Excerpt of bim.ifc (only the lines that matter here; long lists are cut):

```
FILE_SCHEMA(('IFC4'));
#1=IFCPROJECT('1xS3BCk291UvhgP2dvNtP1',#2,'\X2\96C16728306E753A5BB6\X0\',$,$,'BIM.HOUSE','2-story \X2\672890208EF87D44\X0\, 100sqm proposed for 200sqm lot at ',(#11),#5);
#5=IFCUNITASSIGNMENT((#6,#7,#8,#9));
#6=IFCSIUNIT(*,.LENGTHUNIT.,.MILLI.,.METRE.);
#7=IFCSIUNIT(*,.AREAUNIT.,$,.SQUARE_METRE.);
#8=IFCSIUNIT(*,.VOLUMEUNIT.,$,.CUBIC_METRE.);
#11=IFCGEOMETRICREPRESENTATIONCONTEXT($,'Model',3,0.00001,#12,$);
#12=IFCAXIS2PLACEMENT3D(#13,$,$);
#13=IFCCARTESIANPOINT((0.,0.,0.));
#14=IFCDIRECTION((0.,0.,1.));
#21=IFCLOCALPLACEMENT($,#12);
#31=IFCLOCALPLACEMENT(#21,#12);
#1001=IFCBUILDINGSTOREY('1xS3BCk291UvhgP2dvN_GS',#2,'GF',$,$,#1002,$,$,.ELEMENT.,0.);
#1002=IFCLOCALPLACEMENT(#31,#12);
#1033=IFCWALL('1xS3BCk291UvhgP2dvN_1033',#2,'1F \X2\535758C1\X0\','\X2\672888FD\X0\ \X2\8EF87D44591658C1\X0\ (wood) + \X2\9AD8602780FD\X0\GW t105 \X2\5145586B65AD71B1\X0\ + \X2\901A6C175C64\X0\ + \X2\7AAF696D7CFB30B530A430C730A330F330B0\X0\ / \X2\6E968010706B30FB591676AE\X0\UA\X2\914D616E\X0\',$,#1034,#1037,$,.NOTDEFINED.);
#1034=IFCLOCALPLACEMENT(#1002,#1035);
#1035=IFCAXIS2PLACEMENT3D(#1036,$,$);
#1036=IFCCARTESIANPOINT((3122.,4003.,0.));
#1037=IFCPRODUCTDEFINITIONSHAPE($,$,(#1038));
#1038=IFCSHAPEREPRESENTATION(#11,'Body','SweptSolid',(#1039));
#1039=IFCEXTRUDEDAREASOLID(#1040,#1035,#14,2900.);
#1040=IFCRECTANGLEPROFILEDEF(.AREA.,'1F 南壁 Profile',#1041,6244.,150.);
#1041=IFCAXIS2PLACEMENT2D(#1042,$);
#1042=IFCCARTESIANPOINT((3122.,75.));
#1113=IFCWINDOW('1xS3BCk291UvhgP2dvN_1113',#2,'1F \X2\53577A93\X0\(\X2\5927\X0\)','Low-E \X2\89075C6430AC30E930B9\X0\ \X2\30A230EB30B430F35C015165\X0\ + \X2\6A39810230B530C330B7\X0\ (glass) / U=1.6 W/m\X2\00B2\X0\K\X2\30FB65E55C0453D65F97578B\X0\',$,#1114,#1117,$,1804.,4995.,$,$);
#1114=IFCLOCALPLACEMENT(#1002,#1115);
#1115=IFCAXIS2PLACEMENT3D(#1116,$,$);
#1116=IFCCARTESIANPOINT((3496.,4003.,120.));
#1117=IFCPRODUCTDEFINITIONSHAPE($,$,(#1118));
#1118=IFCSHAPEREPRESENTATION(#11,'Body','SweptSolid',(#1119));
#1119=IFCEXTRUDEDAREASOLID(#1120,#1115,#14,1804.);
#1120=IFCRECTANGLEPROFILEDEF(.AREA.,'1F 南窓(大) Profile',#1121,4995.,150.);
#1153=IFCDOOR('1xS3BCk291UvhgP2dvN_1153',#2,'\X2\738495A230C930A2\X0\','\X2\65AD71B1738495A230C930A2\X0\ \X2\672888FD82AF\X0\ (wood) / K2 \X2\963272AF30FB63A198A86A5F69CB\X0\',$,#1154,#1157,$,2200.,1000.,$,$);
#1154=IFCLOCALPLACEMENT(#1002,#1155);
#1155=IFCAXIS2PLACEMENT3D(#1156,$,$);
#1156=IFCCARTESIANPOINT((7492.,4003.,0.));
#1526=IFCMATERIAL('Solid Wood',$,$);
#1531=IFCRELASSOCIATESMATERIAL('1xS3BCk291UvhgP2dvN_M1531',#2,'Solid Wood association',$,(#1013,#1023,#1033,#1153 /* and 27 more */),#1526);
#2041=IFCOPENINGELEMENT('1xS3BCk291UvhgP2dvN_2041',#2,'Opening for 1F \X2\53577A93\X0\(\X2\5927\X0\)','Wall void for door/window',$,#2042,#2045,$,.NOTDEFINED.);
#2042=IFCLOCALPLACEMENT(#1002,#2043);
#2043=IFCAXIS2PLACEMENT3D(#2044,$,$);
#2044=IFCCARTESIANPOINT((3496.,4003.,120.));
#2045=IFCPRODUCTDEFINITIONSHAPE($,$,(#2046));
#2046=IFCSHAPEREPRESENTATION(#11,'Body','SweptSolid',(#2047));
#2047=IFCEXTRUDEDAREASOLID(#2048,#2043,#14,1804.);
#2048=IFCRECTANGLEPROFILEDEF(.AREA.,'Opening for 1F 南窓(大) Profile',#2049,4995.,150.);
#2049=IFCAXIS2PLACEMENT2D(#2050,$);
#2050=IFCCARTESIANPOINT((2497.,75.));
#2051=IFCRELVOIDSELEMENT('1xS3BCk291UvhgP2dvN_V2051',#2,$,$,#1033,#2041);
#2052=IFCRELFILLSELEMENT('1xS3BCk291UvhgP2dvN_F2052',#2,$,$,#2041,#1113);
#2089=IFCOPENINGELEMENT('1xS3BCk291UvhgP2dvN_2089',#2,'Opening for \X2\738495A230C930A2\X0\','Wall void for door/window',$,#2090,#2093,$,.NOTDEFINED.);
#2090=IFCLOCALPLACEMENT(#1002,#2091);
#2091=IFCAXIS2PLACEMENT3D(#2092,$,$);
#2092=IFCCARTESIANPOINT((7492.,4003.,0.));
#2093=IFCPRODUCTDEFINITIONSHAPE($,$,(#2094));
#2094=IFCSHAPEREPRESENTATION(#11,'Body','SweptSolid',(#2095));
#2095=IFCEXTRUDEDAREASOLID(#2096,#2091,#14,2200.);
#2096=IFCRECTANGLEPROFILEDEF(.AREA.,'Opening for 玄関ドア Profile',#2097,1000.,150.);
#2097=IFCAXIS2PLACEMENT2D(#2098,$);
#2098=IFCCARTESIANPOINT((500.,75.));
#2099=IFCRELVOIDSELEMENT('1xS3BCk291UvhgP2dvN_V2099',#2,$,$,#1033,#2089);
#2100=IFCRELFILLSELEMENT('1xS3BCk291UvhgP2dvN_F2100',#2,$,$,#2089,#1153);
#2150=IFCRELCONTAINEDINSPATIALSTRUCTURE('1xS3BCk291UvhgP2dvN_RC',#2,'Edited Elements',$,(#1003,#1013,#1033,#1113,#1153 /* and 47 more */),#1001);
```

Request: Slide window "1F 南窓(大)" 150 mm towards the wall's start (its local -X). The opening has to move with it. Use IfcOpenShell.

```python
import ifcopenshell
import ifcopenshell.api.geometry
import ifcopenshell.util.placement
import ifcopenshell.util.unit

model = ifcopenshell.open("bim.ifc")
unit_scale = ifcopenshell.util.unit.calculate_unit_scale(model)

window = model.by_guid("1xS3BCk291UvhgP2dvN_1113")
opening = window.FillsVoids[0].RelatingOpeningElement
wall = opening.VoidsElements[0].RelatingBuildingElement

wall_matrix = ifcopenshell.util.placement.get_local_placement(wall.ObjectPlacement)
shift = wall_matrix[:3, 0] * -0.15 / unit_scale
before = ifcopenshell.util.placement.get_local_placement(window.ObjectPlacement)[:3, 3].copy()

# The window is not placed relative to its opening, so move both.
for product in (opening, window):
    matrix = ifcopenshell.util.placement.get_local_placement(product.ObjectPlacement)
    matrix[:3, 3] += shift
    ifcopenshell.api.geometry.edit_object_placement(model, product=product, matrix=matrix, is_si=False)

after = ifcopenshell.util.placement.get_local_placement(window.ObjectPlacement)[:3, 3]
print("window moved by", (after - before).round(3) + 0.0)

model.write("bim_rev.ifc")
```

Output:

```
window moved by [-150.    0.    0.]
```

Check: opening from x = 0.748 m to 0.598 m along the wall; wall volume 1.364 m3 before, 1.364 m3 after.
